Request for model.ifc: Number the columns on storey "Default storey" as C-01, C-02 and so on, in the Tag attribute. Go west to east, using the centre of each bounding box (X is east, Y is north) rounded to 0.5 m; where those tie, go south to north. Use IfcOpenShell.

First a look at what the model holds.

```python
import ifcopenshell
import ifcopenshell.util.element
import ifcopenshell.util.placement

model = ifcopenshell.open("model.ifc")
print(model.schema)
storey = next(s for s in model.by_type("IfcBuildingStorey") if s.Name == "Default storey")
columns = [e for e in ifcopenshell.util.element.get_decomposition(storey) if e.is_a("IfcColumn")]
for e in sorted(columns, key=lambda e: e.id()):
    origin = ifcopenshell.util.placement.get_local_placement(e.ObjectPlacement)[:3, 3]
    print(e.id(), e.Tag, e.Name, origin.round(2) + 0.0, sep=" | ")
```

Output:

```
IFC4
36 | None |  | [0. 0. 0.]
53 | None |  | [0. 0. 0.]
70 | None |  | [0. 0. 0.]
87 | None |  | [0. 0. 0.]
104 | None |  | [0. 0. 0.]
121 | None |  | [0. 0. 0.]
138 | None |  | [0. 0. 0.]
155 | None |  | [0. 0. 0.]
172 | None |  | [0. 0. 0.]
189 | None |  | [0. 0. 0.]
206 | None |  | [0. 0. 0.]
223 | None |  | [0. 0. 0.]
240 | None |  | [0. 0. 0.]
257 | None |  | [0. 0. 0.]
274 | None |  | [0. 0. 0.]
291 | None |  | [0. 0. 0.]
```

```python
import ifcopenshell
import ifcopenshell.geom
import ifcopenshell.util.element
import ifcopenshell.util.shape

model = ifcopenshell.open("model.ifc")
settings = ifcopenshell.geom.settings()
settings.set("use-world-coords", True)


def centre(element):
    shape = ifcopenshell.geom.create_shape(settings, element)
    return ifcopenshell.util.shape.get_bbox_centroid(shape.geometry)


storey = next(s for s in model.by_type("IfcBuildingStorey") if s.Name == "Default storey")
columns = [e for e in ifcopenshell.util.element.get_decomposition(storey) if e.is_a("IfcColumn")]

# Insertion points can sit at a corner or the storey origin, so sort by the geometry (in metres).
centres = {e: centre(e) for e in columns}
columns.sort(key=lambda e: (round(centres[e][0] / 0.5), centres[e][1]))

for i, e in enumerate(columns, start=1):
    number = f"C-{i:02d}"
    e.Tag = number
    print(e.id(), number)

model.write("model_v2.ifc")
```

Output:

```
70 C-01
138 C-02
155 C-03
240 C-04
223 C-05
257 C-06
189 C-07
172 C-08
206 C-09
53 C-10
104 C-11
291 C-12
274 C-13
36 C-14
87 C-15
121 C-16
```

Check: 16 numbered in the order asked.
